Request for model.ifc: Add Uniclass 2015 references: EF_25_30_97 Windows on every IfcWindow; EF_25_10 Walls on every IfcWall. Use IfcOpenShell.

First a look at what the model holds.

```python
import ifcopenshell

model = ifcopenshell.open("model.ifc")
print(model.schema)
print("classifications:", [c.Name for c in model.by_type("IfcClassification")])
for ifc_class in ("IfcDoor", "IfcRoof", "IfcStair", "IfcWall", "IfcWindow"):
    print(ifc_class, len(model.by_type(ifc_class)))
```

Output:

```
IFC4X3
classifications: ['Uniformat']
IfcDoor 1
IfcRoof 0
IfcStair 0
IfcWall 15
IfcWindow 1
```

```python
import ifcopenshell
import ifcopenshell.api.classification

model = ifcopenshell.open("model.ifc")

system = ifcopenshell.api.classification.add_classification(model, classification="Uniclass 2015")

codes = {
    "IfcWindow": ("EF_25_30_97", "Windows"),
    "IfcWall": ("EF_25_10", "Walls"),
}
for ifc_class, (code, name) in codes.items():
    products = model.by_type(ifc_class)
    ifcopenshell.api.classification.add_reference(
        model, products=products, classification=system, identification=code, name=name
    )
    print(code, len(products))

model.write("model-out.ifc")
```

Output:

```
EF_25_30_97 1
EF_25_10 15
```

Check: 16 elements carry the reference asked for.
